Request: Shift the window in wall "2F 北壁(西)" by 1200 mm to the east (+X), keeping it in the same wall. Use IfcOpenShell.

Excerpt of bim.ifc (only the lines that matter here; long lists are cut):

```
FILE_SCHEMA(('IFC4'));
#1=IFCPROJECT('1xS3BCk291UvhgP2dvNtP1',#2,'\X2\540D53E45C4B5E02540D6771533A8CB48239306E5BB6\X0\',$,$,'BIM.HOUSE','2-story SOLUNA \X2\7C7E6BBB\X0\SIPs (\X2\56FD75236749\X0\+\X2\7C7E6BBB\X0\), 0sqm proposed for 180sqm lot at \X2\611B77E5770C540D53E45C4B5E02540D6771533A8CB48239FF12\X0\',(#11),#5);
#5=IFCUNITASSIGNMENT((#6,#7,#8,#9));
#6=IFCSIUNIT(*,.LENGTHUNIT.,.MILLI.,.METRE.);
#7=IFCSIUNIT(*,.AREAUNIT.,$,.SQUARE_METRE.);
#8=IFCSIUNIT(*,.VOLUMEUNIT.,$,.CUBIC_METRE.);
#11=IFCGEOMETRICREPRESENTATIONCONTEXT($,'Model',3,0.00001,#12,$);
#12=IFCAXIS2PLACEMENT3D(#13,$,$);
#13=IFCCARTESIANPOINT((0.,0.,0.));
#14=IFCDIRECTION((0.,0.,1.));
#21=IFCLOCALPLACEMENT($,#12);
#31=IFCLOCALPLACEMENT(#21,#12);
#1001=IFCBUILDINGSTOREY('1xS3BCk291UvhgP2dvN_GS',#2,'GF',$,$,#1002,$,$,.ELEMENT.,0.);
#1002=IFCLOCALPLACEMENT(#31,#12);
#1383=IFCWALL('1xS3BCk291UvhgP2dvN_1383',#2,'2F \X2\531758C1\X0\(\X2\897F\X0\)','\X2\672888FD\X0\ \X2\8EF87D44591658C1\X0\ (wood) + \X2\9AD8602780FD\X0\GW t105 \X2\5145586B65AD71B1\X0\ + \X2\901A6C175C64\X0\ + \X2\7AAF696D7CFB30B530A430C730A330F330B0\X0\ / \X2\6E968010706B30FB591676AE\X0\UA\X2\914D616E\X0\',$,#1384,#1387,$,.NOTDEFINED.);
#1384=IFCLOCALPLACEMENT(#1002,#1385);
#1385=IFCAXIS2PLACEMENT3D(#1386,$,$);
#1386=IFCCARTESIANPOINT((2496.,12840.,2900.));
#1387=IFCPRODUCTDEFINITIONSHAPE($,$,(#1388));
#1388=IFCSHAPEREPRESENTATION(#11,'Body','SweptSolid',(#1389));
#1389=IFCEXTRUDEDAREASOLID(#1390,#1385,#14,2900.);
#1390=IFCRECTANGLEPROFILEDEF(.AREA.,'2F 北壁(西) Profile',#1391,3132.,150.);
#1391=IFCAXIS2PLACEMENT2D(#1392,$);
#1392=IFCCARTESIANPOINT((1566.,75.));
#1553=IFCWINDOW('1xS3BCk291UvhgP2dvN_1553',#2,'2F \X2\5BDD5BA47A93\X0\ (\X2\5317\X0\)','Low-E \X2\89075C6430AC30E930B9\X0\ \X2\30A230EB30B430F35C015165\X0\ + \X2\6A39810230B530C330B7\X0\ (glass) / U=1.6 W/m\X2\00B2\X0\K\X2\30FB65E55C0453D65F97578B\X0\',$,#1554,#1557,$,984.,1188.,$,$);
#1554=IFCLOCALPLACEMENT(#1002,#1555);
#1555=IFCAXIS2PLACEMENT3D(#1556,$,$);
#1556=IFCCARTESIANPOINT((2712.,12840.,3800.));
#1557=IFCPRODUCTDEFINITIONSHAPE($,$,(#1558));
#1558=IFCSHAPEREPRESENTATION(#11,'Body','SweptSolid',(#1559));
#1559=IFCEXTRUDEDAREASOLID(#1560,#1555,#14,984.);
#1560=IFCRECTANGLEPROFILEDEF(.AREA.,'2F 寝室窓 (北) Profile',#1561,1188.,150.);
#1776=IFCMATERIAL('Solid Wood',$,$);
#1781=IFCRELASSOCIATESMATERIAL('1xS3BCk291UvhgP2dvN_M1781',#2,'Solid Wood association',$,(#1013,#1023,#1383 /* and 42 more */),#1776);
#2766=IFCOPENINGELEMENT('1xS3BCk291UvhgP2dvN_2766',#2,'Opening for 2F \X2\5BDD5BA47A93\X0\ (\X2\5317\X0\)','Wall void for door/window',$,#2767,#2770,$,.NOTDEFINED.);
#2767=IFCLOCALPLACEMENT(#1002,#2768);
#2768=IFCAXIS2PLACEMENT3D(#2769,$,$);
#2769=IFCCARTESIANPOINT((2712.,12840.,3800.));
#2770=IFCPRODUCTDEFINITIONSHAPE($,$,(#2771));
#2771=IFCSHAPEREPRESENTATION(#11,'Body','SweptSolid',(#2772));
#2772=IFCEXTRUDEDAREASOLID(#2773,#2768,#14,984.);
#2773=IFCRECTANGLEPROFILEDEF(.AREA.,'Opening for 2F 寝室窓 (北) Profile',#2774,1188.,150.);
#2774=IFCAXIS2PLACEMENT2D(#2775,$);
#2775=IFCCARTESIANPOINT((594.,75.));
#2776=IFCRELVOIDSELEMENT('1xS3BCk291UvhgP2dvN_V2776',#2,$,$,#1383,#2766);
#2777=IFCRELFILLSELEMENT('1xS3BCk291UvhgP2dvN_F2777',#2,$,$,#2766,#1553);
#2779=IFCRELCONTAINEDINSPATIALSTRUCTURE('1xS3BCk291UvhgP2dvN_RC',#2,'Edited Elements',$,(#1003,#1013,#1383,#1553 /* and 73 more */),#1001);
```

```python
import ifcopenshell
import ifcopenshell.api.geometry
import ifcopenshell.util.placement
import ifcopenshell.util.unit

model = ifcopenshell.open("bim.ifc")
unit_scale = ifcopenshell.util.unit.calculate_unit_scale(model)

window = model.by_id(1553)
opening = window.FillsVoids[0].RelatingOpeningElement
wall = opening.VoidsElements[0].RelatingBuildingElement

wall_matrix = ifcopenshell.util.placement.get_local_placement(wall.ObjectPlacement)
shift = wall_matrix[:3, 0] * 1.2 / unit_scale
before = ifcopenshell.util.placement.get_local_placement(window.ObjectPlacement)[:3, 3].copy()

# The window is not placed relative to its opening, so move both.
for product in (opening, window):
    matrix = ifcopenshell.util.placement.get_local_placement(product.ObjectPlacement)
    matrix[:3, 3] += shift
    ifcopenshell.api.geometry.edit_object_placement(model, product=product, matrix=matrix, is_si=False)

after = ifcopenshell.util.placement.get_local_placement(window.ObjectPlacement)[:3, 3]
print("window moved by", (after - before).round(3) + 0.0)

model.write("bim-out.ifc")
```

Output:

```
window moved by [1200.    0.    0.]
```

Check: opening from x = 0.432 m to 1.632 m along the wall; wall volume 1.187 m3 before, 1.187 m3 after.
